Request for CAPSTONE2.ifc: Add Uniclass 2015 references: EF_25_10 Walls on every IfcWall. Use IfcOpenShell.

First a look at what the model holds.

```python
import ifcopenshell

model = ifcopenshell.open("CAPSTONE2.ifc")
print(model.schema)
print("classifications:", [c.Name for c in model.by_type("IfcClassification")])
for ifc_class in ("IfcDoor", "IfcRoof", "IfcStair", "IfcWall", "IfcWindow"):
    print(ifc_class, len(model.by_type(ifc_class)))
```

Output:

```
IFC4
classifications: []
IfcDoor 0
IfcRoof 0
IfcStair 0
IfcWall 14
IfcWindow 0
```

```python
import ifcopenshell
import ifcopenshell.api.classification

model = ifcopenshell.open("CAPSTONE2.ifc")

system = ifcopenshell.api.classification.add_classification(model, classification="Uniclass 2015")

codes = {
    "IfcWall": ("EF_25_10", "Walls"),
}
for ifc_class, (code, name) in codes.items():
    products = model.by_type(ifc_class)
    ifcopenshell.api.classification.add_reference(
        model, products=products, classification=system, identification=code, name=name
    )
    print(code, len(products))

model.write("CAPSTONE2_rev.ifc")
```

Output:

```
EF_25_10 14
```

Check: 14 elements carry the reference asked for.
